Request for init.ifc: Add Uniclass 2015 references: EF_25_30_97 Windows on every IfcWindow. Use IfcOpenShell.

First a look at what the model holds.

```python
import ifcopenshell

model = ifcopenshell.open("init.ifc")
print(model.schema)
print("classifications:", [c.Name for c in model.by_type("IfcClassification")])
for ifc_class in ("IfcDoor", "IfcRoof", "IfcStair", "IfcWall", "IfcWindow"):
    print(ifc_class, len(model.by_type(ifc_class)))
```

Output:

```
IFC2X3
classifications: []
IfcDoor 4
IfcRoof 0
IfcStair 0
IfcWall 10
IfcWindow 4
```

```python
import ifcopenshell
import ifcopenshell.api.classification

model = ifcopenshell.open("init.ifc")

# IFC2X3 requires Source and Edition and has no link from the project to the system.
system = model.create_entity("IfcClassification", Source="NBS", Edition="2015", Name="Uniclass 2015")

codes = {
    "IfcWindow": ("EF_25_30_97", "Windows"),
}
for ifc_class, (code, name) in codes.items():
    products = model.by_type(ifc_class)
    ifcopenshell.api.classification.add_reference(
        model, products=products, classification=system, identification=code, name=name
    )
    print(code, len(products))

model.write("init_rev.ifc")
```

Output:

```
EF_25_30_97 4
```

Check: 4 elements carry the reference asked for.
